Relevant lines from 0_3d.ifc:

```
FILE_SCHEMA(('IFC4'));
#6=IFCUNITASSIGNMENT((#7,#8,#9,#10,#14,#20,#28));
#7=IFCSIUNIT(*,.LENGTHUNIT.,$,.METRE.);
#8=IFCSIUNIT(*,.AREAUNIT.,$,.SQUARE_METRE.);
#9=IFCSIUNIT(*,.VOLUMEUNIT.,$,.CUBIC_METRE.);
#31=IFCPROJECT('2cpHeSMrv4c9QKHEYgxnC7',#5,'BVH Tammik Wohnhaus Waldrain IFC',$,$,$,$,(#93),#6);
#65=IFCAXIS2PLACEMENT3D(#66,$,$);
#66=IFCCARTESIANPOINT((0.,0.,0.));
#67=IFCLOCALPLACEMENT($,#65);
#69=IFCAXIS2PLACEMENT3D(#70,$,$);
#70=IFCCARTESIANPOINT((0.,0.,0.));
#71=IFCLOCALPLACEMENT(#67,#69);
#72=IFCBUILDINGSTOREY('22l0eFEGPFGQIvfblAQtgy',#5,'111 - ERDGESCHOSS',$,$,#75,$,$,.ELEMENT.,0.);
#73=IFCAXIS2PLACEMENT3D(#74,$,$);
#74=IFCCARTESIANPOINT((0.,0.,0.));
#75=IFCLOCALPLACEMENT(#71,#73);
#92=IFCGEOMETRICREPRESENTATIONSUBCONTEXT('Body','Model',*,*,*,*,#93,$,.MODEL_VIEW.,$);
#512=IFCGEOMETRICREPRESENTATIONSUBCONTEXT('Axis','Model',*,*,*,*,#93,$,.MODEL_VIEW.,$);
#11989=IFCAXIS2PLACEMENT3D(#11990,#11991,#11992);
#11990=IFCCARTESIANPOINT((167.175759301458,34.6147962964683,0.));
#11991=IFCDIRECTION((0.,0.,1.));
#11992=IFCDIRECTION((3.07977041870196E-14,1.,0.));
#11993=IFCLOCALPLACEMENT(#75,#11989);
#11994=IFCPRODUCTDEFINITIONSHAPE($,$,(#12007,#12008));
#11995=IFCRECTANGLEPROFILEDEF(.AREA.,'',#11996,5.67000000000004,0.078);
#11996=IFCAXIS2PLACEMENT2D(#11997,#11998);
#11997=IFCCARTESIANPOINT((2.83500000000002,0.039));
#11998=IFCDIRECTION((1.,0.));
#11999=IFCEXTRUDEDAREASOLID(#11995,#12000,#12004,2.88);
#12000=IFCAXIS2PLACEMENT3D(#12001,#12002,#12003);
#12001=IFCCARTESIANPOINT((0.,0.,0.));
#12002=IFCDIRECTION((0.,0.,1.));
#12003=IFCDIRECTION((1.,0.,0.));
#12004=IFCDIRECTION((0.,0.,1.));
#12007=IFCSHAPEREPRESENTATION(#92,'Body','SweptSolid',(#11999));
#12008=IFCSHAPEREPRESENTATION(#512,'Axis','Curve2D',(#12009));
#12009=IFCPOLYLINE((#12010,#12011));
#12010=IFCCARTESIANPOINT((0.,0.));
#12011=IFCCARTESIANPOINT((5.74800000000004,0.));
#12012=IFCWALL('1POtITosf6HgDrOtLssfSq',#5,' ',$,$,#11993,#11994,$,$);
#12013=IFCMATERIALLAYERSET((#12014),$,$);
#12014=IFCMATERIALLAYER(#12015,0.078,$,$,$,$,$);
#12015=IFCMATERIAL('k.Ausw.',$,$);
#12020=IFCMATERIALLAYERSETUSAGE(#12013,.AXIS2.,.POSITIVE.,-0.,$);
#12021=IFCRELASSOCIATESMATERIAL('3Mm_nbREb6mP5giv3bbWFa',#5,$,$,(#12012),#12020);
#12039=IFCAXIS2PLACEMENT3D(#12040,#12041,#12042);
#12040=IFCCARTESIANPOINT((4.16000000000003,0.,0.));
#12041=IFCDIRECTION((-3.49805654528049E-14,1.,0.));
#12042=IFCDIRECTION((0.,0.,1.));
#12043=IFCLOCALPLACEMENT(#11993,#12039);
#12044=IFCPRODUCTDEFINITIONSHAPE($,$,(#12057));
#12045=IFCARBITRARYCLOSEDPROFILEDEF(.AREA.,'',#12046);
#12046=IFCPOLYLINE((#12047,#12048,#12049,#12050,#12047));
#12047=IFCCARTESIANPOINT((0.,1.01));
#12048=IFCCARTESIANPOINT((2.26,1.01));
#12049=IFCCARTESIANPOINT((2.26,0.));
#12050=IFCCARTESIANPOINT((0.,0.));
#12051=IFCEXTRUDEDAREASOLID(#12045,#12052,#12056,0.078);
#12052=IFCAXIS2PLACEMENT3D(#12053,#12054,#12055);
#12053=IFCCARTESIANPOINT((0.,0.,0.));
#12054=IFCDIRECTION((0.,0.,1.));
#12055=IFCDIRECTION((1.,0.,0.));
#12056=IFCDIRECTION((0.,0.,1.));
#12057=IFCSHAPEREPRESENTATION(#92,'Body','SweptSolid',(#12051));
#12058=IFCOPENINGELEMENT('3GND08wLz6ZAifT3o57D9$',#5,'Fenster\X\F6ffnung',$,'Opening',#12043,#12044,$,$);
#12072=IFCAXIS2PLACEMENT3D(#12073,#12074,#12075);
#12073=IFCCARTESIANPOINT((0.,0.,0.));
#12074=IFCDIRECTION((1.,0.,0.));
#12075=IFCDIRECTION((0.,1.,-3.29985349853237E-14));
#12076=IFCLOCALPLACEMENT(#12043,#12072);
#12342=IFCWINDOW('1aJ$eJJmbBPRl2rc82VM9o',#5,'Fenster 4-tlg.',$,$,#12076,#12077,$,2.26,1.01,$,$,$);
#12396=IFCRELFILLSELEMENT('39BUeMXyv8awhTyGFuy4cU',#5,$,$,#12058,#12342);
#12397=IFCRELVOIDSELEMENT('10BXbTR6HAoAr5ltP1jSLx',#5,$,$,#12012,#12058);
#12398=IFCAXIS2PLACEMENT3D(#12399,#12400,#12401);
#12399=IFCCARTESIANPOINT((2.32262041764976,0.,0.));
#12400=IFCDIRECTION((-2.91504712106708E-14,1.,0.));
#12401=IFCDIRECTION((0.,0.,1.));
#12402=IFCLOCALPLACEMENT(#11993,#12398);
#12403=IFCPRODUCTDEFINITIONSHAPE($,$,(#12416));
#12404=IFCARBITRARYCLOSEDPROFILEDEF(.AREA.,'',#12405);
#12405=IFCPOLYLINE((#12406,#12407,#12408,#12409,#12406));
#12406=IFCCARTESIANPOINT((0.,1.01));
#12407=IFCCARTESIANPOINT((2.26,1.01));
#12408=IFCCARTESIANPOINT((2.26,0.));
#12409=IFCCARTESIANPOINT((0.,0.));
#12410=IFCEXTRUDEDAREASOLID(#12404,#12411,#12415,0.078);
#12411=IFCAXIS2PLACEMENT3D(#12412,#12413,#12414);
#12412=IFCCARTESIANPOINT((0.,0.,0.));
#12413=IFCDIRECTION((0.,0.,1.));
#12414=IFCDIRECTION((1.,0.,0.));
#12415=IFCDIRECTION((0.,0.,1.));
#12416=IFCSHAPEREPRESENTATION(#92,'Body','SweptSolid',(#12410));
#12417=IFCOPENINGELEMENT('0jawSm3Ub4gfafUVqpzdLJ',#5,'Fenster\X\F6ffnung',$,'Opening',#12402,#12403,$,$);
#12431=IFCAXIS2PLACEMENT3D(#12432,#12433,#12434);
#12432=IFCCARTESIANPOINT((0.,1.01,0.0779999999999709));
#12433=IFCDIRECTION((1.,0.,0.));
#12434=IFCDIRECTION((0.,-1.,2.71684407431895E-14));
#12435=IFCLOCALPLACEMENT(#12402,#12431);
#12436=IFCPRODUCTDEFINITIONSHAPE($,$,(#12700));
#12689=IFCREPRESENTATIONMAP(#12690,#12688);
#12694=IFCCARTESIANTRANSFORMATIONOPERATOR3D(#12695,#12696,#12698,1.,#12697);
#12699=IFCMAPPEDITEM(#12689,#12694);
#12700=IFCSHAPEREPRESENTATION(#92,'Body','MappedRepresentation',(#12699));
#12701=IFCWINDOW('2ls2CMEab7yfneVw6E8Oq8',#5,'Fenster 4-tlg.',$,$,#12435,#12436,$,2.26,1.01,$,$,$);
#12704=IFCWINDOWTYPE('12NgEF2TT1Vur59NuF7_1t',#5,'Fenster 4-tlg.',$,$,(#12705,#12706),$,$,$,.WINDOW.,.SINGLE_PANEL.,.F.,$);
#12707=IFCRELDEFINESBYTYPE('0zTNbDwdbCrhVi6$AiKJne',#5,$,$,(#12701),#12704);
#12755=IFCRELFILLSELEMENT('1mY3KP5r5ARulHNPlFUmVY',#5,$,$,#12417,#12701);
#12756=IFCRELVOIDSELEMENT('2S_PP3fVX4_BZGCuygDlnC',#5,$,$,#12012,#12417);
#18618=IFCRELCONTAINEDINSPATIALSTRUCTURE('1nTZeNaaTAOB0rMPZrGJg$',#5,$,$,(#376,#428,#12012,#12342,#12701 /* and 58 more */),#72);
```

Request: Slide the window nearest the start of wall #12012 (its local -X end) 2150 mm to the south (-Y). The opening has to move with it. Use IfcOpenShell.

```python
import ifcopenshell
import ifcopenshell.api.geometry
import ifcopenshell.util.placement

model = ifcopenshell.open("0_3d.ifc")

window = model.by_guid("2ls2CMEab7yfneVw6E8Oq8")
opening = window.FillsVoids[0].RelatingOpeningElement
wall = opening.VoidsElements[0].RelatingBuildingElement

wall_matrix = ifcopenshell.util.placement.get_local_placement(wall.ObjectPlacement)
shift = wall_matrix[:3, 0] * -2.15
before = ifcopenshell.util.placement.get_local_placement(window.ObjectPlacement)[:3, 3].copy()

# The window is placed relative to its opening, so it follows when the opening moves.
matrix = ifcopenshell.util.placement.get_local_placement(opening.ObjectPlacement)
matrix[:3, 3] += shift
ifcopenshell.api.geometry.edit_object_placement(
    model, product=opening, matrix=matrix, is_si=False, should_transform_children=True
)

after = ifcopenshell.util.placement.get_local_placement(window.ObjectPlacement)[:3, 3]
print("window moved by", (after - before).round(3) + 0.0)

model.write("0_3d-out.ifc")
```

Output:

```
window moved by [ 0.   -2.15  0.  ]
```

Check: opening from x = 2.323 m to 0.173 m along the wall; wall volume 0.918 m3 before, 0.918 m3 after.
